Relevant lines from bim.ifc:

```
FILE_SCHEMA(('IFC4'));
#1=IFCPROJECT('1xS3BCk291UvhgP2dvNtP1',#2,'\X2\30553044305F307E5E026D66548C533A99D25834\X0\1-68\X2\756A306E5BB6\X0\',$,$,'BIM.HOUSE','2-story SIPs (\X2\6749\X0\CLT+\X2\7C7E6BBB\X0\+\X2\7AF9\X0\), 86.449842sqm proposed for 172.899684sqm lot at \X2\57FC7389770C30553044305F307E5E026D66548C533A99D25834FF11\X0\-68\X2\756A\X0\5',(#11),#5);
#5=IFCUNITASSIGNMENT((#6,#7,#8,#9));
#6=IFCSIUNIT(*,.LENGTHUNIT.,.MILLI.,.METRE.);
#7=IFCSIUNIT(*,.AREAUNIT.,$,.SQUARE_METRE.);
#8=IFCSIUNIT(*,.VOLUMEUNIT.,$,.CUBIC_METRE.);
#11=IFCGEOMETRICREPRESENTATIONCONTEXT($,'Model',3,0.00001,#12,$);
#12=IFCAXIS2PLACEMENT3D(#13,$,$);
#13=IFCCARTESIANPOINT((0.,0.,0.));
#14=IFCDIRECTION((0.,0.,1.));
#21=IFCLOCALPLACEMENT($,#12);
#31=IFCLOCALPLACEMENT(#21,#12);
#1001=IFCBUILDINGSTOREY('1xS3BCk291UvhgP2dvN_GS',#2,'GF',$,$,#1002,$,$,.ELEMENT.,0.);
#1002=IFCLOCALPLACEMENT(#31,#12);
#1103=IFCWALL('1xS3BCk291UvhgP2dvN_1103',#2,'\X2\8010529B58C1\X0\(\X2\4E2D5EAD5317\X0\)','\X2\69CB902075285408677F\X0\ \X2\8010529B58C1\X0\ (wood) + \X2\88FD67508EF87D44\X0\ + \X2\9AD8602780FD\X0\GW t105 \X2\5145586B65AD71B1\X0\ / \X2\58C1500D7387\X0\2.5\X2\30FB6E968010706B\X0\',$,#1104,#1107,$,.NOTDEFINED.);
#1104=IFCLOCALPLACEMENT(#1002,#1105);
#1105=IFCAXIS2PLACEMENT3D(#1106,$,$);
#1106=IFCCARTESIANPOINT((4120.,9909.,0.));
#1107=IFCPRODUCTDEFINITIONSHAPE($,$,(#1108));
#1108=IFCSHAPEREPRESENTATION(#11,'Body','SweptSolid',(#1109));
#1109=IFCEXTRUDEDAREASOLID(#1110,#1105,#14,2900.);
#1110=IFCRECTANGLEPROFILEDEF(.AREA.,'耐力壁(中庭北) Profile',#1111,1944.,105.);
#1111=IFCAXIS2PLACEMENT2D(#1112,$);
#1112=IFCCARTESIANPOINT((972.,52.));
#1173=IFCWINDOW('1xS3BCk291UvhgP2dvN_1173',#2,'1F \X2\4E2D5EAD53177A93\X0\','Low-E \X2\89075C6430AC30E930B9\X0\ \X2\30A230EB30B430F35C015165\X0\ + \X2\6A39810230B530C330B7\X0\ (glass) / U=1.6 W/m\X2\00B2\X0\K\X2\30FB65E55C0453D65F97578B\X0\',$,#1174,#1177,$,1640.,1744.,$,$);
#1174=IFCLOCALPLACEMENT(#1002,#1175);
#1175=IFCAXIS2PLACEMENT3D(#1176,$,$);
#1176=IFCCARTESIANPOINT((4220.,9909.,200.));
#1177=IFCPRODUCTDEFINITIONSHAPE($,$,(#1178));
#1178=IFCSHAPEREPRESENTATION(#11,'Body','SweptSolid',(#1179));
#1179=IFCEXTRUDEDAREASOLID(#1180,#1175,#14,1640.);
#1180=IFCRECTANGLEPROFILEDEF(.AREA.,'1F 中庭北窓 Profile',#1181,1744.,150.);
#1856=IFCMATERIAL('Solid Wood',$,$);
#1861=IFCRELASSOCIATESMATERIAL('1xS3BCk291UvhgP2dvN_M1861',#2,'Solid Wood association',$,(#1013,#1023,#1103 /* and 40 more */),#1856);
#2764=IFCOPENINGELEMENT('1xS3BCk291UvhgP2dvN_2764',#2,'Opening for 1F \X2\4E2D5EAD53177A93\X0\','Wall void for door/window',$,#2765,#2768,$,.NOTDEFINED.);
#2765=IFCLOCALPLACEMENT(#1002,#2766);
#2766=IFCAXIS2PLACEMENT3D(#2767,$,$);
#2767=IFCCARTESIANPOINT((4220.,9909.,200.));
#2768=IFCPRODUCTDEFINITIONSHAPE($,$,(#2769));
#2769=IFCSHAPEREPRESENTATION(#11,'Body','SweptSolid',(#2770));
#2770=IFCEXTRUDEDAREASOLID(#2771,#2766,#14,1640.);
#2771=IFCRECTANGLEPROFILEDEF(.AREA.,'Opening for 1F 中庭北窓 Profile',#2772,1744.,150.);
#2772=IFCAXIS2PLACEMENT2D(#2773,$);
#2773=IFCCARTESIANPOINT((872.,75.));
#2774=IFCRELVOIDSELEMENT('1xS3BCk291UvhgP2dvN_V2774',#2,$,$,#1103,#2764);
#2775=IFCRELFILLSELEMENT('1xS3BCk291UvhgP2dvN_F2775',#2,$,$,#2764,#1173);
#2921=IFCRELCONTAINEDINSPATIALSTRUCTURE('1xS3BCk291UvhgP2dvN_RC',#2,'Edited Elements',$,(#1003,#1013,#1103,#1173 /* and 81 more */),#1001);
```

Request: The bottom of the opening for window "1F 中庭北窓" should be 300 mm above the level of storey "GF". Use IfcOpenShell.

```python
import numpy as np
import ifcopenshell
import ifcopenshell.api.geometry
import ifcopenshell.geom
import ifcopenshell.util.element
import ifcopenshell.util.placement
import ifcopenshell.util.shape
import ifcopenshell.util.unit

model = ifcopenshell.open("bim.ifc")
unit_scale = ifcopenshell.util.unit.calculate_unit_scale(model)

window = model.by_guid("1xS3BCk291UvhgP2dvN_1173")
opening = window.FillsVoids[0].RelatingOpeningElement
storey = ifcopenshell.util.element.get_container(window, ifc_class="IfcBuildingStorey")
level = ifcopenshell.util.placement.get_local_placement(storey.ObjectPlacement)[2, 3]

# The opening's origin need not be at the sill, so measure its lowest point.
shape = ifcopenshell.geom.create_shape(ifcopenshell.geom.settings(), opening)
bottom = ifcopenshell.util.shape.get_shape_bottom_elevation(shape, shape.geometry) / unit_scale
dz = level + 0.3 / unit_scale - bottom

shift = np.array([0.0, 0.0, dz])
# The window is not placed relative to its opening, so move both.
for product in (opening, window):
    matrix = ifcopenshell.util.placement.get_local_placement(product.ObjectPlacement)
    matrix[:3, 3] += shift
    ifcopenshell.api.geometry.edit_object_placement(model, product=product, matrix=matrix, is_si=False)

print(f"moved by {dz * unit_scale:+.3f} m")

model.write("bim_v2.ifc")
```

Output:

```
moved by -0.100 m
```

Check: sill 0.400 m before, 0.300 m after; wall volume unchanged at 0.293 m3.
